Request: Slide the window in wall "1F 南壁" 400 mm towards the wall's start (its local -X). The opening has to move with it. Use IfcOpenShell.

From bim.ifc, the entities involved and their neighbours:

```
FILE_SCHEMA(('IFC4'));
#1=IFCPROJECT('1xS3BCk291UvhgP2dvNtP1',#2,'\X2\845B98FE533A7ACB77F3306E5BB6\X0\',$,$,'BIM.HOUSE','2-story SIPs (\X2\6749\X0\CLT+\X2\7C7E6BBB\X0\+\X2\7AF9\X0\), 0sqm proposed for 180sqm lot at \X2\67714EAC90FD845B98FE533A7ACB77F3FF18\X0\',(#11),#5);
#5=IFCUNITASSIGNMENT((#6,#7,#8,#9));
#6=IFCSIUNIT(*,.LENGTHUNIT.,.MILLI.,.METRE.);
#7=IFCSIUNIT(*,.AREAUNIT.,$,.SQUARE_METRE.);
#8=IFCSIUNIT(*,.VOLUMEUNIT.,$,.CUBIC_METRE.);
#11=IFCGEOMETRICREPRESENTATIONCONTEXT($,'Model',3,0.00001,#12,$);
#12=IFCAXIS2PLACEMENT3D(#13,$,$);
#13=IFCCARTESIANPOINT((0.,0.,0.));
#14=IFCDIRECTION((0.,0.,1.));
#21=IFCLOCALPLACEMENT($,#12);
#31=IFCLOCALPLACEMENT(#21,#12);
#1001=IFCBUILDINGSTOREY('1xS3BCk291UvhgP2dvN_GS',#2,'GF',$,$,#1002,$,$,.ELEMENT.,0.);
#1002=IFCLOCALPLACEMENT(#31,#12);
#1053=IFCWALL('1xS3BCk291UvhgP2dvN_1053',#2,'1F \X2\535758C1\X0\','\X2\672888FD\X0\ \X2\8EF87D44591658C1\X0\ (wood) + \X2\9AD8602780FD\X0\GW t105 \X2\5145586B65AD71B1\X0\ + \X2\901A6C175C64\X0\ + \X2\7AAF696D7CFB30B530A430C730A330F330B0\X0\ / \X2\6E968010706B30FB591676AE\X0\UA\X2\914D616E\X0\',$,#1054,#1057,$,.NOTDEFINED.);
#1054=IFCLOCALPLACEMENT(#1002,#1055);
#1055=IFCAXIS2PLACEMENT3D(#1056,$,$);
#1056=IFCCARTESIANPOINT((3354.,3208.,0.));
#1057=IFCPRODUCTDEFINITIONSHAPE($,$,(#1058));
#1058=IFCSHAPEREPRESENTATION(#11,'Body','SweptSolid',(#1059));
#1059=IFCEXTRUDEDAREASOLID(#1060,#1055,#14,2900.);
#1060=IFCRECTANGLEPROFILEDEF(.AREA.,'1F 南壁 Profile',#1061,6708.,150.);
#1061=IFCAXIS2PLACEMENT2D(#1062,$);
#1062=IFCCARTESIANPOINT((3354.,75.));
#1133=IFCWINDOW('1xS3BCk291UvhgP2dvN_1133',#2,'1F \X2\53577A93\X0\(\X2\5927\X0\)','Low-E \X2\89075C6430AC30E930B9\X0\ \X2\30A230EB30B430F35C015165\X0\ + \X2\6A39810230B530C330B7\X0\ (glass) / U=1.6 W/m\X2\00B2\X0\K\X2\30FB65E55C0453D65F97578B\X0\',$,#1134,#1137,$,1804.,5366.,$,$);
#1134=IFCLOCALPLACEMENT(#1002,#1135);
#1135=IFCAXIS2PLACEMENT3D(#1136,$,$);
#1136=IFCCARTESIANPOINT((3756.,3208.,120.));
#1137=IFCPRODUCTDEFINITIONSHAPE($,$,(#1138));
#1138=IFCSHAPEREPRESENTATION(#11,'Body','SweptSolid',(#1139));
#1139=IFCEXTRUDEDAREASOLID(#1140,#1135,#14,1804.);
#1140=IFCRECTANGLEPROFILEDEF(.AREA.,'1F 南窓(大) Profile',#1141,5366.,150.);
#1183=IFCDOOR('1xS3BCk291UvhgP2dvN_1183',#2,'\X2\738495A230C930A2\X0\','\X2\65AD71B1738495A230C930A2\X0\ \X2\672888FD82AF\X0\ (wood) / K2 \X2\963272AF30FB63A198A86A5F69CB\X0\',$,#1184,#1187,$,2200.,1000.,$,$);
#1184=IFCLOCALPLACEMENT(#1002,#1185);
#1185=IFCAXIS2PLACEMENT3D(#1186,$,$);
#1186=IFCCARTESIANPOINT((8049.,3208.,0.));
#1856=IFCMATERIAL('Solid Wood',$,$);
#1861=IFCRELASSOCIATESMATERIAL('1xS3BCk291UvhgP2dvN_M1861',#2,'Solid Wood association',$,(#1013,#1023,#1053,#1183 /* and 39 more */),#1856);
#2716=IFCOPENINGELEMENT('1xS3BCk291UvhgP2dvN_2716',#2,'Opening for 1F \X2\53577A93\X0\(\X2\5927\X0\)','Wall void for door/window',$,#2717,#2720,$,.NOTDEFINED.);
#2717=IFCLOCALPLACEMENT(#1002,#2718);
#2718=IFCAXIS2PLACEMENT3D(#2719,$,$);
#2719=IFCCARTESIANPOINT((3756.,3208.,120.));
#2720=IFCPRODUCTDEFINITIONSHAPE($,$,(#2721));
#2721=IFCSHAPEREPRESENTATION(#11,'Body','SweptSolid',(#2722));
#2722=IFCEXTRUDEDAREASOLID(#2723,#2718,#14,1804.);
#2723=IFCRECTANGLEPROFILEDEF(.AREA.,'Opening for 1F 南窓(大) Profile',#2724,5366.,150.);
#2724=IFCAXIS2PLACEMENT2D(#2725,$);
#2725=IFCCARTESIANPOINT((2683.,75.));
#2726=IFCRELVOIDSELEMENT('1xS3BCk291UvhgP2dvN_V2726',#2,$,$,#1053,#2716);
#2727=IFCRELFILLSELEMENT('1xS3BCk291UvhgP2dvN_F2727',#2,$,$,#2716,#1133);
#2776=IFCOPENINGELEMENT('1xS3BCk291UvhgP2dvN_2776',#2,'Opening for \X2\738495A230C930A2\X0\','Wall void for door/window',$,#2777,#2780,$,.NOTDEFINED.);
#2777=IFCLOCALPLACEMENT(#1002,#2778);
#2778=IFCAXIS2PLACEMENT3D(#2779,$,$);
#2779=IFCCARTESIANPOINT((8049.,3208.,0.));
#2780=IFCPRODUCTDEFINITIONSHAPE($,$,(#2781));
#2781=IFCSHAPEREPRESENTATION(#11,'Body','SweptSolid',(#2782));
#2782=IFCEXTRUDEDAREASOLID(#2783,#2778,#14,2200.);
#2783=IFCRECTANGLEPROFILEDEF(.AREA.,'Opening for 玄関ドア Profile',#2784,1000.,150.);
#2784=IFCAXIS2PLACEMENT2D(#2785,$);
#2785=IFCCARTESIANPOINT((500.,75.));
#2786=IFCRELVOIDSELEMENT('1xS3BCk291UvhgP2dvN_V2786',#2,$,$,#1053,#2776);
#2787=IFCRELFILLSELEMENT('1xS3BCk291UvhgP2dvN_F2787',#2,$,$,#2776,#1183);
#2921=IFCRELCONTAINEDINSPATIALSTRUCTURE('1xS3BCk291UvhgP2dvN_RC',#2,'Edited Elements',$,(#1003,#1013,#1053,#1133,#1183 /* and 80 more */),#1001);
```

```python
import ifcopenshell
import ifcopenshell.api.geometry
import ifcopenshell.util.placement
import ifcopenshell.util.unit

model = ifcopenshell.open("bim.ifc")
unit_scale = ifcopenshell.util.unit.calculate_unit_scale(model)

window = model.by_guid("1xS3BCk291UvhgP2dvN_1133")
opening = window.FillsVoids[0].RelatingOpeningElement
wall = opening.VoidsElements[0].RelatingBuildingElement

wall_matrix = ifcopenshell.util.placement.get_local_placement(wall.ObjectPlacement)
shift = wall_matrix[:3, 0] * -0.4 / unit_scale
before = ifcopenshell.util.placement.get_local_placement(window.ObjectPlacement)[:3, 3].copy()

# The window is not placed relative to its opening, so move both.
for product in (opening, window):
    matrix = ifcopenshell.util.placement.get_local_placement(product.ObjectPlacement)
    matrix[:3, 3] += shift
    ifcopenshell.api.geometry.edit_object_placement(model, product=product, matrix=matrix, is_si=False)

after = ifcopenshell.util.placement.get_local_placement(window.ObjectPlacement)[:3, 3]
print("window moved by", (after - before).round(3) + 0.0)

model.write("bim_updated.ifc")
```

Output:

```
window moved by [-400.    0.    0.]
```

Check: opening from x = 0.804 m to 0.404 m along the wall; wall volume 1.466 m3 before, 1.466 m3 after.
